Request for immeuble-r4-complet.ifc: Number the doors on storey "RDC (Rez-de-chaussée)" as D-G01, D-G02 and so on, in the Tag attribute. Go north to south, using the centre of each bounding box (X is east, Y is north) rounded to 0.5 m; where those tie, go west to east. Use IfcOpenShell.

First a look at what the model holds.

```python
import ifcopenshell
import ifcopenshell.util.element
import ifcopenshell.util.placement

model = ifcopenshell.open("immeuble-r4-complet.ifc")
print(model.schema)
storey = next(s for s in model.by_type("IfcBuildingStorey") if s.Name == "RDC (Rez-de-chaussée)")
doors = [e for e in ifcopenshell.util.element.get_decomposition(storey) if e.is_a("IfcDoor")]
for e in sorted(doors, key=lambda e: e.id()):
    origin = ifcopenshell.util.placement.get_local_placement(e.ObjectPlacement)[:3, 3]
    print(e.id(), e.Tag, e.Name, origin.round(2) + 0.0, sep=" | ")
```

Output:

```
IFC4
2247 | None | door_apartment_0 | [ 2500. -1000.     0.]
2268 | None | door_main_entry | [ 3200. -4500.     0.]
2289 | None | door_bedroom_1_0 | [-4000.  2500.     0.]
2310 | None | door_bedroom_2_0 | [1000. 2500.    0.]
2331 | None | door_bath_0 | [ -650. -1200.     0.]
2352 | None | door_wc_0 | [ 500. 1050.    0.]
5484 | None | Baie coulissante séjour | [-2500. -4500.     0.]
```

```python
import ifcopenshell
import ifcopenshell.geom
import ifcopenshell.util.element
import ifcopenshell.util.shape

model = ifcopenshell.open("immeuble-r4-complet.ifc")
settings = ifcopenshell.geom.settings()
settings.set("use-world-coords", True)


def centre(element):
    shape = ifcopenshell.geom.create_shape(settings, element)
    return ifcopenshell.util.shape.get_bbox_centroid(shape.geometry)


storey = next(s for s in model.by_type("IfcBuildingStorey") if s.Name == "RDC (Rez-de-chaussée)")
doors = [e for e in ifcopenshell.util.element.get_decomposition(storey) if e.is_a("IfcDoor")]

# Insertion points can sit at a corner or the storey origin, so sort by the geometry (in metres).
centres = {e: centre(e) for e in doors}
doors.sort(key=lambda e: (-round(centres[e][1] / 0.5), centres[e][0]))

for i, e in enumerate(doors, start=1):
    number = f"D-G{i:02d}"
    e.Tag = number
    print(e.id(), number)

model.write("immeuble-r4-complet_v2.ifc")
```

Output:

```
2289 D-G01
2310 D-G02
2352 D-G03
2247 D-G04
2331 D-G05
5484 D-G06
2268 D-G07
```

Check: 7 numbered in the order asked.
